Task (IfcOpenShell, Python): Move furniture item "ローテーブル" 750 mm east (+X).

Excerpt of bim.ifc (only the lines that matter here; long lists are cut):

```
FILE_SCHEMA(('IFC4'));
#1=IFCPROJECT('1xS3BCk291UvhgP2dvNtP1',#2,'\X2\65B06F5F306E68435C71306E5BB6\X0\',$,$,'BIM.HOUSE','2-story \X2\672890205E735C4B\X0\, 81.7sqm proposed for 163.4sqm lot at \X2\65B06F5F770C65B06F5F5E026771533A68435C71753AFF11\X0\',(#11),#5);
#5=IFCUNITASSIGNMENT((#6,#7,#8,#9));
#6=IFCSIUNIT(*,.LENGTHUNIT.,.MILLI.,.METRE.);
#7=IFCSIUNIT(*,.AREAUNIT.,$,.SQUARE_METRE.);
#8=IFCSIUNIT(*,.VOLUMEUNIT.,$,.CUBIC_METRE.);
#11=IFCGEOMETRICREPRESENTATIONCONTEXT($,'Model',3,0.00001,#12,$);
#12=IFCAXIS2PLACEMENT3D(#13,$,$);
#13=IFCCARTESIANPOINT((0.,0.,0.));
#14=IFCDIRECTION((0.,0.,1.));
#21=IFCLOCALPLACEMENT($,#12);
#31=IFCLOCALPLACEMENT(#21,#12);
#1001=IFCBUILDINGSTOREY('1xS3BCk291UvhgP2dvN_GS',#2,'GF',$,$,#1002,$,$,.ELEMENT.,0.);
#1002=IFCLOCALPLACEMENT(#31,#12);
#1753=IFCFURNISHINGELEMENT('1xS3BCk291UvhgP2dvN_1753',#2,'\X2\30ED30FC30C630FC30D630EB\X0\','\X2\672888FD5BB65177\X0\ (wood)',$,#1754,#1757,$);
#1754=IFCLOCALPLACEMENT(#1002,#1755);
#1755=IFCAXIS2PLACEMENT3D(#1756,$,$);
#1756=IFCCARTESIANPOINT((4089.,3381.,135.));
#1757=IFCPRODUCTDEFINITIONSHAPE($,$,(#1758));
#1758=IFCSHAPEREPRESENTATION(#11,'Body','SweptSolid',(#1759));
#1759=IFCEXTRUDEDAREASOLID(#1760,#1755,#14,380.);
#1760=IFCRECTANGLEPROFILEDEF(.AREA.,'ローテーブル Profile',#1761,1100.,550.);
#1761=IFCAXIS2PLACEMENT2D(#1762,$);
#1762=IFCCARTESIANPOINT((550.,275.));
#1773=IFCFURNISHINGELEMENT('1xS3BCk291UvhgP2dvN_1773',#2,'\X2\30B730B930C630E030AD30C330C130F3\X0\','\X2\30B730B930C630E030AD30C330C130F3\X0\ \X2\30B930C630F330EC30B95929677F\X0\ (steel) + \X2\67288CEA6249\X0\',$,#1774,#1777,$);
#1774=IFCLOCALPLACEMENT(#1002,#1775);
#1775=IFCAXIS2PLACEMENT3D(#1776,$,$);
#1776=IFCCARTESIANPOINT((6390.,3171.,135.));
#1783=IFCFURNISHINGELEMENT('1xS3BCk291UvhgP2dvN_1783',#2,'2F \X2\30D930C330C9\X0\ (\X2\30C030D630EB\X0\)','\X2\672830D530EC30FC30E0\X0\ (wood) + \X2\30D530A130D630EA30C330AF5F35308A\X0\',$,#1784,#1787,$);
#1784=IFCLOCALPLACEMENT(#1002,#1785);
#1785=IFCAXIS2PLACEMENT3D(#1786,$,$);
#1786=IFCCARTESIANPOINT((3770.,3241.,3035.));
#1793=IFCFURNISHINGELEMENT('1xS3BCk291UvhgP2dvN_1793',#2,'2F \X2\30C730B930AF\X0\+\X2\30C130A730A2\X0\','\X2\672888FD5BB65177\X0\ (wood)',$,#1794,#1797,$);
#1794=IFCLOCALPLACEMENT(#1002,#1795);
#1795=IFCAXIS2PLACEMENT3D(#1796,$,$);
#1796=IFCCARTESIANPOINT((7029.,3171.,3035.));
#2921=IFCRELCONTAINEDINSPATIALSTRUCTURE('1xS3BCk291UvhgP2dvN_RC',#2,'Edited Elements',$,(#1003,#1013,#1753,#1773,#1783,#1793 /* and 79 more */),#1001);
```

```python
import ifcopenshell
import ifcopenshell.api.geometry
import ifcopenshell.util.placement
import ifcopenshell.util.unit

model = ifcopenshell.open("bim.ifc")
unit_scale = ifcopenshell.util.unit.calculate_unit_scale(model)

item = model.by_guid("1xS3BCk291UvhgP2dvN_1753")
matrix = ifcopenshell.util.placement.get_local_placement(item.ObjectPlacement)
matrix[0, 3] += 0.75 / unit_scale
ifcopenshell.api.geometry.edit_object_placement(model, product=item, matrix=matrix, is_si=False)

print(ifcopenshell.util.placement.get_local_placement(item.ObjectPlacement).round(3) + 0.0)

model.write("bim-out.ifc")
```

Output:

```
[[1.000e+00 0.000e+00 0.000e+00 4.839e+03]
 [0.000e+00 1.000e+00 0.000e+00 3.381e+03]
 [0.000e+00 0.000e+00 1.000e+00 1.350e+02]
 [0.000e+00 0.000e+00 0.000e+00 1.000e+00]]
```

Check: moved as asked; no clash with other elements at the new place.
